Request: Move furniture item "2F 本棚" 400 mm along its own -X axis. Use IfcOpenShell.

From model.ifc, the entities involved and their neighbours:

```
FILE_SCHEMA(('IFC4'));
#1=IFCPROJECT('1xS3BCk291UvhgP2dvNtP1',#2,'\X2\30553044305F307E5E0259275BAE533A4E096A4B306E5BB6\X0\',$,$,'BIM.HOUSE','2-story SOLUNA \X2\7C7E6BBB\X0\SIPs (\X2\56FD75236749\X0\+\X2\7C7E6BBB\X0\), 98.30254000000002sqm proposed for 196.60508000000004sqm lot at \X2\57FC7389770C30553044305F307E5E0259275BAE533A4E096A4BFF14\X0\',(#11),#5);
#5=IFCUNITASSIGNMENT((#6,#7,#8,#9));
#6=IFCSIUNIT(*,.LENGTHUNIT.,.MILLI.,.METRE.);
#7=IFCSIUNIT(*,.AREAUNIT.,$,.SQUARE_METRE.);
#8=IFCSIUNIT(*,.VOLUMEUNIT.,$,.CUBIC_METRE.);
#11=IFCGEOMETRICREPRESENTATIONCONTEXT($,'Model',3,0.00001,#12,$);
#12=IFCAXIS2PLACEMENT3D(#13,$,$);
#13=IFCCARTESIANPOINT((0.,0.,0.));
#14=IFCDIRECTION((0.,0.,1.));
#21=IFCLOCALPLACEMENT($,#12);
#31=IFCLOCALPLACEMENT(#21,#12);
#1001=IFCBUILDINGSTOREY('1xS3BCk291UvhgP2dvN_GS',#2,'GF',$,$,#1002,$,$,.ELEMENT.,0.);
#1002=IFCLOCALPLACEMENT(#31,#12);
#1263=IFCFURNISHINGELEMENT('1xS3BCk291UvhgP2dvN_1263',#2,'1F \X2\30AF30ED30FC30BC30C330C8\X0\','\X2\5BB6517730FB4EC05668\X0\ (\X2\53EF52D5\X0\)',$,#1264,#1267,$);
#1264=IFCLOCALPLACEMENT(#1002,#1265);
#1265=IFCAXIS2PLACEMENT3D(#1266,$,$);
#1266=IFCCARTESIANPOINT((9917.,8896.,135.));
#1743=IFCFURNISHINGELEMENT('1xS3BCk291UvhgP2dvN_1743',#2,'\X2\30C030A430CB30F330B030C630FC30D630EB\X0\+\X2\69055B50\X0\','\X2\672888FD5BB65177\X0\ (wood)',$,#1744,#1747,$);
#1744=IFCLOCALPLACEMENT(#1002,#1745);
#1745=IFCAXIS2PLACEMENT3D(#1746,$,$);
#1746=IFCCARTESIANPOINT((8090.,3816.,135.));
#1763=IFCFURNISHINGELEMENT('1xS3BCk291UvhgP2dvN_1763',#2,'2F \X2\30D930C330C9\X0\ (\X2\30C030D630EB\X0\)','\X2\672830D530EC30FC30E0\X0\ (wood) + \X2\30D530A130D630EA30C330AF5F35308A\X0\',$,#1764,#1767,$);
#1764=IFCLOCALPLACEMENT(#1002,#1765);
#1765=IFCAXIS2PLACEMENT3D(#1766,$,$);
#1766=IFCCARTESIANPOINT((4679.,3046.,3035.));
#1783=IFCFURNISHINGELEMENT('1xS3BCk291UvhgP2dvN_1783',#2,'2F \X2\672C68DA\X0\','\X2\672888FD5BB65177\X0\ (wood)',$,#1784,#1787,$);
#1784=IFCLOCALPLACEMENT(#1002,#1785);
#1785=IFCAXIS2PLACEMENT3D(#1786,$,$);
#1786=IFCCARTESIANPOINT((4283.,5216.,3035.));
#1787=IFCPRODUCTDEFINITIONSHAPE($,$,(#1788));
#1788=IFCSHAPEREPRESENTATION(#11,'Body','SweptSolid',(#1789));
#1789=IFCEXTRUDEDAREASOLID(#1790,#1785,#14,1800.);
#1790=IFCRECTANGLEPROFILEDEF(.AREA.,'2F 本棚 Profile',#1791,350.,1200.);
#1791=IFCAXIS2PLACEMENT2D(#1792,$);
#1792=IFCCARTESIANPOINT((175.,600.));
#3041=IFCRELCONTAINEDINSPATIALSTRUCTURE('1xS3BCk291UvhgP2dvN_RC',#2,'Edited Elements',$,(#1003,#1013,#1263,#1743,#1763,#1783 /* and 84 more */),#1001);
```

```python
import ifcopenshell
import ifcopenshell.api.geometry
import ifcopenshell.util.placement

model = ifcopenshell.open("model.ifc")

item = model.by_guid("1xS3BCk291UvhgP2dvN_1783")
matrix = ifcopenshell.util.placement.get_local_placement(item.ObjectPlacement)
matrix[:3, 3] -= matrix[:3, 0] * 400.0
ifcopenshell.api.geometry.edit_object_placement(model, product=item, matrix=matrix, is_si=False)

print(ifcopenshell.util.placement.get_local_placement(item.ObjectPlacement).round(3) + 0.0)

model.write("model_updated.ifc")
```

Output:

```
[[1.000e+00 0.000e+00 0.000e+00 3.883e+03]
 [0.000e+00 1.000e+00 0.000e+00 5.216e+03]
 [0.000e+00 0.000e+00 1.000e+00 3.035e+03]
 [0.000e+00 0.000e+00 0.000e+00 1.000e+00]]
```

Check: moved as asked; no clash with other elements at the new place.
